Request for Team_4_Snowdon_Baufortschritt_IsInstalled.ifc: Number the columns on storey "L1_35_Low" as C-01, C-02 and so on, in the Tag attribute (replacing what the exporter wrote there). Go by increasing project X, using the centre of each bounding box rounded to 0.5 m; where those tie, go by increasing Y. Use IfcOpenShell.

First a look at what the model holds.

```python
import ifcopenshell
import ifcopenshell.util.element
import ifcopenshell.util.placement

model = ifcopenshell.open("Team_4_Snowdon_Baufortschritt_IsInstalled.ifc")
print(model.schema)
storey = next(s for s in model.by_type("IfcBuildingStorey") if s.Name == "L1_35_Low")
columns = [e for e in ifcopenshell.util.element.get_decomposition(storey) if e.is_a("IfcColumn")]
for e in sorted(columns, key=lambda e: e.id()):
    origin = ifcopenshell.util.placement.get_local_placement(e.ObjectPlacement)[:3, 3]
    print(e.id(), e.Tag, e.Name, origin.round(2) + 0.0, sep=" | ")
```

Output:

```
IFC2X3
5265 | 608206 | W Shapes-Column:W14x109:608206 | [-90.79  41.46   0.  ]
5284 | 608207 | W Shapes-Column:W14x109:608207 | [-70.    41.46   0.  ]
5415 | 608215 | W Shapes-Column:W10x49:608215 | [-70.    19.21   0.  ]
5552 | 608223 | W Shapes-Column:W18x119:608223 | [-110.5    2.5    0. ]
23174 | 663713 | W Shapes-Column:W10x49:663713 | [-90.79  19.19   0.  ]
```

```python
import ifcopenshell
import ifcopenshell.geom
import ifcopenshell.util.element
import ifcopenshell.util.shape

model = ifcopenshell.open("Team_4_Snowdon_Baufortschritt_IsInstalled.ifc")
settings = ifcopenshell.geom.settings()
settings.set("use-world-coords", True)


def centre(element):
    shape = ifcopenshell.geom.create_shape(settings, element)
    return ifcopenshell.util.shape.get_bbox_centroid(shape.geometry)


storey = next(s for s in model.by_type("IfcBuildingStorey") if s.Name == "L1_35_Low")
columns = [e for e in ifcopenshell.util.element.get_decomposition(storey) if e.is_a("IfcColumn")]

# Insertion points can sit at a corner or the storey origin, so sort by the geometry (in metres).
centres = {e: centre(e) for e in columns}
columns.sort(key=lambda e: (round(centres[e][0] / 0.5), centres[e][1]))

for i, e in enumerate(columns, start=1):
    number = f"C-{i:02d}"
    e.Tag = number
    print(e.id(), number)

model.write("Team_4_Snowdon_Baufortschritt_IsInstalled_edited.ifc")
```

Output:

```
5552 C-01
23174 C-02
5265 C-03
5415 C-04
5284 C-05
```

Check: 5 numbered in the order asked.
